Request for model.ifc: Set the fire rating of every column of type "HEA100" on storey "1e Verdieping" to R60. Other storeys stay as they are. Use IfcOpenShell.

First a look at what the model holds.

```python
import ifcopenshell
import ifcopenshell.util.element

model = ifcopenshell.open("model.ifc")
print(model.schema)
storey = next(s for s in model.by_type("IfcBuildingStorey") if s.Name == "1e Verdieping")
columns = [e for e in ifcopenshell.util.element.get_decomposition(storey) if e.is_a("IfcColumn")]
seen = {}
for e in columns:
    element_type = ifcopenshell.util.element.get_type(e)
    key = (element_type.Name if element_type != e and element_type else None, ifcopenshell.util.element.get_pset(e, "Pset_ColumnCommon", "FireRating"))
    seen[key] = seen.get(key, 0) + 1
for (name, value), count in sorted(seen.items(), key=str):
    print(count, "x", name, "|", value)
```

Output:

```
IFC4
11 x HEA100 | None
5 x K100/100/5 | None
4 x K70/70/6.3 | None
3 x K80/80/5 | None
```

```python
import ifcopenshell
import ifcopenshell.api.pset
import ifcopenshell.util.element

model = ifcopenshell.open("model.ifc")

storey = next(s for s in model.by_type("IfcBuildingStorey") if s.Name == "1e Verdieping")
columns = [e for e in ifcopenshell.util.element.get_decomposition(storey) if e.is_a("IfcColumn")]

count = 0
for e in columns:
    element_type = ifcopenshell.util.element.get_type(e)
    if element_type in (None, e) or element_type.Name != "HEA100":
        continue
    # add_pset returns the element's existing set when there is one.
    pset = ifcopenshell.api.pset.add_pset(model, product=e, name="Pset_ColumnCommon")
    ifcopenshell.api.pset.edit_pset(model, pset=pset, properties={"FireRating": "R60"})
    count += 1

print(count, "columns updated")

model.write("model_updated.ifc")
```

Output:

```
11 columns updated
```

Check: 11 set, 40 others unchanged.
